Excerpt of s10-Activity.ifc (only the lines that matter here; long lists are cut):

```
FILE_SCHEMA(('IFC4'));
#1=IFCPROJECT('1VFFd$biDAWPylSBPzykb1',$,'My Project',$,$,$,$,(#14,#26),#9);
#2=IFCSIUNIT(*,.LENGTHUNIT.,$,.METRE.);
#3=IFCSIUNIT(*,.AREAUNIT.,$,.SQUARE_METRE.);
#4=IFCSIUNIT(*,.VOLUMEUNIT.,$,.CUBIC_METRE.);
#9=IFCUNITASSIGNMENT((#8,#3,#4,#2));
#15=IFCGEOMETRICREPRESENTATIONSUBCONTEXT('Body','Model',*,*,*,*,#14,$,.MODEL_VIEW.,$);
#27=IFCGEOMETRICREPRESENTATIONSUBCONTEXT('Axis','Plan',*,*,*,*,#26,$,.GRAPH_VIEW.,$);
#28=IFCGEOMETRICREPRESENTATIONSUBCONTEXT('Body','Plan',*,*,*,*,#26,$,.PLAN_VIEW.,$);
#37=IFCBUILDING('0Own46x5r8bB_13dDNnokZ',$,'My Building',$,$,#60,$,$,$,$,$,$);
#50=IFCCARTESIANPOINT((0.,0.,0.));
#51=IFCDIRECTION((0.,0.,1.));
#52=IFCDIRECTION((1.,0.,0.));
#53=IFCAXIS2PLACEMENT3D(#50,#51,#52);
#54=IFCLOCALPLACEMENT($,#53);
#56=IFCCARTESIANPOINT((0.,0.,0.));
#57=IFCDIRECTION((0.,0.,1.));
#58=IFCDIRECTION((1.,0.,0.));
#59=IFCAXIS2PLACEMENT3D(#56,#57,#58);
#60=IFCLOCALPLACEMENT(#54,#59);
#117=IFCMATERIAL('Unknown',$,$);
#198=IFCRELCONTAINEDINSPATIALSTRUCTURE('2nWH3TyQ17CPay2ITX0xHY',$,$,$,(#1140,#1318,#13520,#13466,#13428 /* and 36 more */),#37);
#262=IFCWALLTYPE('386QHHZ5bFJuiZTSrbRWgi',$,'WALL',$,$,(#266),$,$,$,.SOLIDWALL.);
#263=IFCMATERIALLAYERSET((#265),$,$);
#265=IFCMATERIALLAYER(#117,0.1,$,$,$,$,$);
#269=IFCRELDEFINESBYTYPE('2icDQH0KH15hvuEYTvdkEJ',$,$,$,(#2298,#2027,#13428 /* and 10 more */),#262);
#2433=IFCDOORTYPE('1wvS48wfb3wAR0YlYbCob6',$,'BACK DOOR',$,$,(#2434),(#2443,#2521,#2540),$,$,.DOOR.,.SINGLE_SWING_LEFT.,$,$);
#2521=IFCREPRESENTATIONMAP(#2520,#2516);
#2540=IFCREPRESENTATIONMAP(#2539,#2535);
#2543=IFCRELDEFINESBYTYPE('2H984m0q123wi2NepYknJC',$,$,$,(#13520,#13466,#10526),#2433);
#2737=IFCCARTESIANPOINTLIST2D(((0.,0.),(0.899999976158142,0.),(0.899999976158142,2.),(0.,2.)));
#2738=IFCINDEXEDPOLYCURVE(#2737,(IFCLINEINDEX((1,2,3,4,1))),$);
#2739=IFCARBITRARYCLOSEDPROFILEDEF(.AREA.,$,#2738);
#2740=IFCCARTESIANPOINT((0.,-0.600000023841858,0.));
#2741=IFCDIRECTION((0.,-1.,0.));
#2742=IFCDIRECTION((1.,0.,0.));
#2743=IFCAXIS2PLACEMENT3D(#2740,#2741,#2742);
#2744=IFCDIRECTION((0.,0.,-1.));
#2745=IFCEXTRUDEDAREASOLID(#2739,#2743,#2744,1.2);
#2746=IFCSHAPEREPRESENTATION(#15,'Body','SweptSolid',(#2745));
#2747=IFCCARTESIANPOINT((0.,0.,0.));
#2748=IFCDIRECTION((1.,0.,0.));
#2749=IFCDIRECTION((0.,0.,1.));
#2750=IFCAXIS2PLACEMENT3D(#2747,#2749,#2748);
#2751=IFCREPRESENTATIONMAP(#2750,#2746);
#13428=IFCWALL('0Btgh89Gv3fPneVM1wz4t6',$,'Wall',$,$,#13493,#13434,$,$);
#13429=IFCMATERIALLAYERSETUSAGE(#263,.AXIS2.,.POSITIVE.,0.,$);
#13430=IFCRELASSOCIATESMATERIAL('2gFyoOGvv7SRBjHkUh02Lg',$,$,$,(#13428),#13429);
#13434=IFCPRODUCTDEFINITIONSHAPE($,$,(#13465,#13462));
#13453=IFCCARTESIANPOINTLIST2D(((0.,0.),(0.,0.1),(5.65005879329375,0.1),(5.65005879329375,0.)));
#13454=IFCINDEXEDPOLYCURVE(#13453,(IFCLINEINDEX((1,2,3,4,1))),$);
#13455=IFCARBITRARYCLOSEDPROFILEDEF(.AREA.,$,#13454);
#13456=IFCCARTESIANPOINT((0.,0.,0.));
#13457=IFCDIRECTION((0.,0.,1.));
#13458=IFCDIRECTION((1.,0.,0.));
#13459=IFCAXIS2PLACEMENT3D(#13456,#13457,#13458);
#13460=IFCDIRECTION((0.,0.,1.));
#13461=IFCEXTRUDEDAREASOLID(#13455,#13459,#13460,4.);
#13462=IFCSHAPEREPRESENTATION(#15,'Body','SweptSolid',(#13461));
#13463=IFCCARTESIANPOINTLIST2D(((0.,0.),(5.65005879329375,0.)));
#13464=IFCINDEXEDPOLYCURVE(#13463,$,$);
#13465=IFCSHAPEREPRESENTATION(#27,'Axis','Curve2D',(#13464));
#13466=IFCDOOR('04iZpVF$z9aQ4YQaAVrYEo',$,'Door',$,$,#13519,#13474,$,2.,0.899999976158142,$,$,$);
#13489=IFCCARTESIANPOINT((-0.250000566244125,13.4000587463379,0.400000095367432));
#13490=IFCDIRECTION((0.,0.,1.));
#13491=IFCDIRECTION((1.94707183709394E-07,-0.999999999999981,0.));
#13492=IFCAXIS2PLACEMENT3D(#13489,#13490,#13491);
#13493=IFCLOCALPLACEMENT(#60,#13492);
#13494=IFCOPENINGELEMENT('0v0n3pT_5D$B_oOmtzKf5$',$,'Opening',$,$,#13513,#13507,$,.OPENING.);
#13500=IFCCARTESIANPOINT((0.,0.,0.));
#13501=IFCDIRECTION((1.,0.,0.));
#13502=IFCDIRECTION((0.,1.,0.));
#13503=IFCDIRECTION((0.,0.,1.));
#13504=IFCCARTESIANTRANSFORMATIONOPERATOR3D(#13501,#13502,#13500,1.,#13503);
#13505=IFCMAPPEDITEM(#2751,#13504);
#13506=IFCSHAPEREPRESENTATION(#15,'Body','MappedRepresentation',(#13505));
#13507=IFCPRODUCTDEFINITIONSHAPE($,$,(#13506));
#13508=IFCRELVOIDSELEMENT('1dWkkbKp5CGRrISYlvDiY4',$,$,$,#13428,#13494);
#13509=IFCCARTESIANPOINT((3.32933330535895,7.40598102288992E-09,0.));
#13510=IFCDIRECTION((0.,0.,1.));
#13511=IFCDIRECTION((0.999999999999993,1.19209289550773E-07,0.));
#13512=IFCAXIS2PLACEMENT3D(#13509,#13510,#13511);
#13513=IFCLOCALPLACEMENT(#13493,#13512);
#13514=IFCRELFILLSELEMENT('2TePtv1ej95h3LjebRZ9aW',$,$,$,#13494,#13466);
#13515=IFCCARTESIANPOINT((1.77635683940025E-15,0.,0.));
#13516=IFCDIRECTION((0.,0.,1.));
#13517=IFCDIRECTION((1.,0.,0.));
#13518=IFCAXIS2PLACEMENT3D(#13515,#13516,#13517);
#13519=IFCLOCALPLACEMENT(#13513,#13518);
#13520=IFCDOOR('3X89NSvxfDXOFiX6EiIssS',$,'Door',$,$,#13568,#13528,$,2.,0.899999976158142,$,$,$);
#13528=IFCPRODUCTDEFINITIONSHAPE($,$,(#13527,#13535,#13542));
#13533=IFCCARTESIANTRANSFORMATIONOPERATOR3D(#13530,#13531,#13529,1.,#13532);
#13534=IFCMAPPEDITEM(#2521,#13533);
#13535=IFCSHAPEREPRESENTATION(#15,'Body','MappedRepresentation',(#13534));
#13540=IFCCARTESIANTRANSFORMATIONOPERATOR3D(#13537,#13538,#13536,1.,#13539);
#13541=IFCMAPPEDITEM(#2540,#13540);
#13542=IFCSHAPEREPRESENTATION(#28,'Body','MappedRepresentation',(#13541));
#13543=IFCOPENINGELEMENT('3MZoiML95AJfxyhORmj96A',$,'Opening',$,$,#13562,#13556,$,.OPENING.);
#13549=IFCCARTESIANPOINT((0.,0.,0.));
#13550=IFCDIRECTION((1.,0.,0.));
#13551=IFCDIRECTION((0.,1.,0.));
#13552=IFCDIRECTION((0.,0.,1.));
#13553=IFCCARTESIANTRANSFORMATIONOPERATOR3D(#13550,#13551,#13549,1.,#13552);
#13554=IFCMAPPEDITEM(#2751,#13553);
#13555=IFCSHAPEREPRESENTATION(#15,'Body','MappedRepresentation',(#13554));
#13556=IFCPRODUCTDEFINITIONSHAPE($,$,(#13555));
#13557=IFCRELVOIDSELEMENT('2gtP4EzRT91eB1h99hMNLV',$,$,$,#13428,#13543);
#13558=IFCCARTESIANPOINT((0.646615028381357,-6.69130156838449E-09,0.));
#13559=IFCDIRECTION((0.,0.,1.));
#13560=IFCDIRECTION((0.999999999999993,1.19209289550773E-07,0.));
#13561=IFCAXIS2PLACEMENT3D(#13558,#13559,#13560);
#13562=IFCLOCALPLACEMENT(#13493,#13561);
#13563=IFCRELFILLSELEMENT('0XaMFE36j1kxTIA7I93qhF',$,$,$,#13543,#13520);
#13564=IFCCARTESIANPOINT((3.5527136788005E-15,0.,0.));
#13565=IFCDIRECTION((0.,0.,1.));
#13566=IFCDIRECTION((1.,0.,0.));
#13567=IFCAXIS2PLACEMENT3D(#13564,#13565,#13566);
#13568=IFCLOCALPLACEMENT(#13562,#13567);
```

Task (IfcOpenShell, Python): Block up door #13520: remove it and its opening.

```python
import ifcopenshell
import ifcopenshell.api.feature
import ifcopenshell.api.root
import ifcopenshell.geom
import ifcopenshell.util.shape

model = ifcopenshell.open("s10-Activity.ifc")
settings = ifcopenshell.geom.settings()


def volume(element):
    """Net volume in cubic metres, openings subtracted."""
    shape = ifcopenshell.geom.create_shape(settings, element)
    return ifcopenshell.util.shape.get_volume(shape.geometry)


door = model.by_id(13520)
opening = door.FillsVoids[0].RelatingOpeningElement
wall = opening.VoidsElements[0].RelatingBuildingElement
before = volume(wall)

ifcopenshell.api.root.remove_product(model, product=door)
ifcopenshell.api.feature.remove_feature(model, feature=opening)

after = volume(wall)

print(f"wall volume {before:.3f} -> {after:.3f} m3")

model.write("s10-Activity_edited.ifc")
```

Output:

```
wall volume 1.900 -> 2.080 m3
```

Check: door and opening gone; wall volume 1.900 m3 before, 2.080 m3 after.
